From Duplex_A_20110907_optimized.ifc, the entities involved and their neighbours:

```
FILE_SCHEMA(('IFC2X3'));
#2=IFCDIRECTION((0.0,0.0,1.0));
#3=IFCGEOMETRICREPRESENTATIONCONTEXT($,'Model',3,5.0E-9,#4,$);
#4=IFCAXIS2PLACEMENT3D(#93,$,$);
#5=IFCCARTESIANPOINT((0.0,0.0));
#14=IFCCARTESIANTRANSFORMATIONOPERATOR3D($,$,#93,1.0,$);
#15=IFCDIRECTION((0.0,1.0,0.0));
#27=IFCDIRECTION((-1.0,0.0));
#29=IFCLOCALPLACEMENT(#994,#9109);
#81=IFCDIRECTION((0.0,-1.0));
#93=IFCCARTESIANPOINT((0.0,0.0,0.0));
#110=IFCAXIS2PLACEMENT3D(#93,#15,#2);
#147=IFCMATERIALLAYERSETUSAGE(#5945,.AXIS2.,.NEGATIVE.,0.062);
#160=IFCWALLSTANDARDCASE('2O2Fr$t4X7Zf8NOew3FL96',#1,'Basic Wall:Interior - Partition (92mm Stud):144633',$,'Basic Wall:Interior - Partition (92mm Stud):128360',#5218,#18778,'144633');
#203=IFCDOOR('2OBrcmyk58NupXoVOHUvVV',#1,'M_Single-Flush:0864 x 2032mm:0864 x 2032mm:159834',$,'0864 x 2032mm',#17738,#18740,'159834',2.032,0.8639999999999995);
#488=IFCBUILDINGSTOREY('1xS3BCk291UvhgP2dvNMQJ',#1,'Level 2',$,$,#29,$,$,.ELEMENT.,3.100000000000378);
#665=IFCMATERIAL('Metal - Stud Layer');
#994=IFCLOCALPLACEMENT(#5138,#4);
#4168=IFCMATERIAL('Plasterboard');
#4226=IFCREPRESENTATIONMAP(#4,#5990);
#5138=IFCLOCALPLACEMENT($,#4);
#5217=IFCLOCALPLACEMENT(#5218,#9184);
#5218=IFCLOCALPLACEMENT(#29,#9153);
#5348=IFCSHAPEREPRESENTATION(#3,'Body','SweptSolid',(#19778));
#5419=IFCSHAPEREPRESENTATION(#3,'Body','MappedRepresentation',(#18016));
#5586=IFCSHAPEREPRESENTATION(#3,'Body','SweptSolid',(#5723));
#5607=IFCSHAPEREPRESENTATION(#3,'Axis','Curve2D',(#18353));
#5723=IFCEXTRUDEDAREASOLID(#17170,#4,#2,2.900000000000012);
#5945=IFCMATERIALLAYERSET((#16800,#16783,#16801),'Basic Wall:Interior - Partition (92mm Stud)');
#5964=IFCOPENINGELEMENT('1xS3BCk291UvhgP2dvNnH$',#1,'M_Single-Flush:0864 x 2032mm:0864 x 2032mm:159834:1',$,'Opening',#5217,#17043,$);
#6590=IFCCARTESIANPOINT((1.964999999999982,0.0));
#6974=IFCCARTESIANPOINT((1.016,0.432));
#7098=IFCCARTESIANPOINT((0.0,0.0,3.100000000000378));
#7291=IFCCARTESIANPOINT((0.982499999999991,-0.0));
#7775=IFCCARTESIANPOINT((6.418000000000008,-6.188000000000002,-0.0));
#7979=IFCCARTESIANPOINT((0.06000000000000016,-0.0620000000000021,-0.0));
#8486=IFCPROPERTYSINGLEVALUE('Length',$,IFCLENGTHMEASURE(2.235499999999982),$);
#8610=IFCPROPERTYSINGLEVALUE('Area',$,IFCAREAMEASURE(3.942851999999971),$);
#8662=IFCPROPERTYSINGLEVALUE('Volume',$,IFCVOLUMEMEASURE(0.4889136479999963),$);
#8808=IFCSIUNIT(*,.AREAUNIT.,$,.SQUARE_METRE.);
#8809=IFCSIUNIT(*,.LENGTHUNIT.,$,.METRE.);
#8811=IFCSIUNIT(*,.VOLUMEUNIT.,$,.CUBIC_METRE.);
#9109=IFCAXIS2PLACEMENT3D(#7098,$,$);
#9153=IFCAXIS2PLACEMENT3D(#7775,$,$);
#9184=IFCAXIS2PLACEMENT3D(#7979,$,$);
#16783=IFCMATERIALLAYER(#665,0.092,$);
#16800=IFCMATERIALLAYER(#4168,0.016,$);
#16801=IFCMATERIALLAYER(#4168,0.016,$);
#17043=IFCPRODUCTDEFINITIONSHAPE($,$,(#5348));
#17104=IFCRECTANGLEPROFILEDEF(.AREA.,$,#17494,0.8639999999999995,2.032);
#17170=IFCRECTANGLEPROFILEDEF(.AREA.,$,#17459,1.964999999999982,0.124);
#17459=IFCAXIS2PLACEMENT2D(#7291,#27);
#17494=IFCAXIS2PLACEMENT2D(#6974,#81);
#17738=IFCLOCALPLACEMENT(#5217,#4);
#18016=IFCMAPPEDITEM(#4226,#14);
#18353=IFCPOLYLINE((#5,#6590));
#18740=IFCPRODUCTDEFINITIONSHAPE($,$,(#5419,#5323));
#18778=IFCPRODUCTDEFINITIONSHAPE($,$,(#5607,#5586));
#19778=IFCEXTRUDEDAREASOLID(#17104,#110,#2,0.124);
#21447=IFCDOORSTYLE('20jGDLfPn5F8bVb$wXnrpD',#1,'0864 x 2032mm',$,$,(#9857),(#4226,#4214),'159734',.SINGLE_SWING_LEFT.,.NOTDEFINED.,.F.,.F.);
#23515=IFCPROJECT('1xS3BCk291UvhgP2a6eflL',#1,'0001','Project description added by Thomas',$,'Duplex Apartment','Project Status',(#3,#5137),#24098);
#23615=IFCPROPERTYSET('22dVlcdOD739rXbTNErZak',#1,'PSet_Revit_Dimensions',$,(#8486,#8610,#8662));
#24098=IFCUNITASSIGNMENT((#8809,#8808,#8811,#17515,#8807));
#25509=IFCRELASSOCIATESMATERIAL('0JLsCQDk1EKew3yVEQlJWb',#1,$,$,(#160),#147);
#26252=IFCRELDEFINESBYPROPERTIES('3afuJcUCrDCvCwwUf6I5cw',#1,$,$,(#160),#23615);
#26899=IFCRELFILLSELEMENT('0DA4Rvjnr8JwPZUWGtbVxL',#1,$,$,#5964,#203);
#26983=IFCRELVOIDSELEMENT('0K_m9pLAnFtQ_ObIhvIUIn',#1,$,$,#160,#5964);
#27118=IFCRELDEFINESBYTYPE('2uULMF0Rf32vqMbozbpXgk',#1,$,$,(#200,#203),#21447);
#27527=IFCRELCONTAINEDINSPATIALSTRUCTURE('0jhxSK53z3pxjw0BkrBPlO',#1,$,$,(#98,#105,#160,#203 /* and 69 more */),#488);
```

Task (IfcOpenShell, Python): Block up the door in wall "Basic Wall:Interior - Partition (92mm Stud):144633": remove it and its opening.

```python
import ifcopenshell
import ifcopenshell.api.feature
import ifcopenshell.api.pset
import ifcopenshell.api.root
import ifcopenshell.geom
import ifcopenshell.util.element
import ifcopenshell.util.shape
import ifcopenshell.util.unit

model = ifcopenshell.open("Duplex_A_20110907_optimized.ifc")
area_scale = ifcopenshell.util.unit.calculate_unit_scale(model, "AREAUNIT")
volume_scale = ifcopenshell.util.unit.calculate_unit_scale(model, "VOLUMEUNIT")
settings = ifcopenshell.geom.settings()


def volume(element):
    """Net volume in cubic metres, openings subtracted."""
    shape = ifcopenshell.geom.create_shape(settings, element)
    return ifcopenshell.util.shape.get_volume(shape.geometry)


door = model.by_id(203)
opening = door.FillsVoids[0].RelatingOpeningElement
wall = opening.VoidsElements[0].RelatingBuildingElement
before = volume(wall)

ifcopenshell.api.root.remove_product(model, product=door)
ifcopenshell.api.feature.remove_feature(model, feature=opening)

after = volume(wall)
thickness = 0.124  # wall thickness in metres

# Update the wall's stored quantities.
pset = model.by_id(ifcopenshell.util.element.get_pset(wall, "PSet_Revit_Dimensions", should_inherit=False)["id"])
ifcopenshell.api.pset.edit_pset(model, pset=pset, properties={
    "Area": model.create_entity("IfcAreaMeasure", after / thickness / area_scale),
    "Volume": model.create_entity("IfcVolumeMeasure", after / volume_scale),
})

print(f"wall volume {before:.3f} -> {after:.3f} m3")

model.write("Duplex_A_20110907_optimized_v2.ifc")
```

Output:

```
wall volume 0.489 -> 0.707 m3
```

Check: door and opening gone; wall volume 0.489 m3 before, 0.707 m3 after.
